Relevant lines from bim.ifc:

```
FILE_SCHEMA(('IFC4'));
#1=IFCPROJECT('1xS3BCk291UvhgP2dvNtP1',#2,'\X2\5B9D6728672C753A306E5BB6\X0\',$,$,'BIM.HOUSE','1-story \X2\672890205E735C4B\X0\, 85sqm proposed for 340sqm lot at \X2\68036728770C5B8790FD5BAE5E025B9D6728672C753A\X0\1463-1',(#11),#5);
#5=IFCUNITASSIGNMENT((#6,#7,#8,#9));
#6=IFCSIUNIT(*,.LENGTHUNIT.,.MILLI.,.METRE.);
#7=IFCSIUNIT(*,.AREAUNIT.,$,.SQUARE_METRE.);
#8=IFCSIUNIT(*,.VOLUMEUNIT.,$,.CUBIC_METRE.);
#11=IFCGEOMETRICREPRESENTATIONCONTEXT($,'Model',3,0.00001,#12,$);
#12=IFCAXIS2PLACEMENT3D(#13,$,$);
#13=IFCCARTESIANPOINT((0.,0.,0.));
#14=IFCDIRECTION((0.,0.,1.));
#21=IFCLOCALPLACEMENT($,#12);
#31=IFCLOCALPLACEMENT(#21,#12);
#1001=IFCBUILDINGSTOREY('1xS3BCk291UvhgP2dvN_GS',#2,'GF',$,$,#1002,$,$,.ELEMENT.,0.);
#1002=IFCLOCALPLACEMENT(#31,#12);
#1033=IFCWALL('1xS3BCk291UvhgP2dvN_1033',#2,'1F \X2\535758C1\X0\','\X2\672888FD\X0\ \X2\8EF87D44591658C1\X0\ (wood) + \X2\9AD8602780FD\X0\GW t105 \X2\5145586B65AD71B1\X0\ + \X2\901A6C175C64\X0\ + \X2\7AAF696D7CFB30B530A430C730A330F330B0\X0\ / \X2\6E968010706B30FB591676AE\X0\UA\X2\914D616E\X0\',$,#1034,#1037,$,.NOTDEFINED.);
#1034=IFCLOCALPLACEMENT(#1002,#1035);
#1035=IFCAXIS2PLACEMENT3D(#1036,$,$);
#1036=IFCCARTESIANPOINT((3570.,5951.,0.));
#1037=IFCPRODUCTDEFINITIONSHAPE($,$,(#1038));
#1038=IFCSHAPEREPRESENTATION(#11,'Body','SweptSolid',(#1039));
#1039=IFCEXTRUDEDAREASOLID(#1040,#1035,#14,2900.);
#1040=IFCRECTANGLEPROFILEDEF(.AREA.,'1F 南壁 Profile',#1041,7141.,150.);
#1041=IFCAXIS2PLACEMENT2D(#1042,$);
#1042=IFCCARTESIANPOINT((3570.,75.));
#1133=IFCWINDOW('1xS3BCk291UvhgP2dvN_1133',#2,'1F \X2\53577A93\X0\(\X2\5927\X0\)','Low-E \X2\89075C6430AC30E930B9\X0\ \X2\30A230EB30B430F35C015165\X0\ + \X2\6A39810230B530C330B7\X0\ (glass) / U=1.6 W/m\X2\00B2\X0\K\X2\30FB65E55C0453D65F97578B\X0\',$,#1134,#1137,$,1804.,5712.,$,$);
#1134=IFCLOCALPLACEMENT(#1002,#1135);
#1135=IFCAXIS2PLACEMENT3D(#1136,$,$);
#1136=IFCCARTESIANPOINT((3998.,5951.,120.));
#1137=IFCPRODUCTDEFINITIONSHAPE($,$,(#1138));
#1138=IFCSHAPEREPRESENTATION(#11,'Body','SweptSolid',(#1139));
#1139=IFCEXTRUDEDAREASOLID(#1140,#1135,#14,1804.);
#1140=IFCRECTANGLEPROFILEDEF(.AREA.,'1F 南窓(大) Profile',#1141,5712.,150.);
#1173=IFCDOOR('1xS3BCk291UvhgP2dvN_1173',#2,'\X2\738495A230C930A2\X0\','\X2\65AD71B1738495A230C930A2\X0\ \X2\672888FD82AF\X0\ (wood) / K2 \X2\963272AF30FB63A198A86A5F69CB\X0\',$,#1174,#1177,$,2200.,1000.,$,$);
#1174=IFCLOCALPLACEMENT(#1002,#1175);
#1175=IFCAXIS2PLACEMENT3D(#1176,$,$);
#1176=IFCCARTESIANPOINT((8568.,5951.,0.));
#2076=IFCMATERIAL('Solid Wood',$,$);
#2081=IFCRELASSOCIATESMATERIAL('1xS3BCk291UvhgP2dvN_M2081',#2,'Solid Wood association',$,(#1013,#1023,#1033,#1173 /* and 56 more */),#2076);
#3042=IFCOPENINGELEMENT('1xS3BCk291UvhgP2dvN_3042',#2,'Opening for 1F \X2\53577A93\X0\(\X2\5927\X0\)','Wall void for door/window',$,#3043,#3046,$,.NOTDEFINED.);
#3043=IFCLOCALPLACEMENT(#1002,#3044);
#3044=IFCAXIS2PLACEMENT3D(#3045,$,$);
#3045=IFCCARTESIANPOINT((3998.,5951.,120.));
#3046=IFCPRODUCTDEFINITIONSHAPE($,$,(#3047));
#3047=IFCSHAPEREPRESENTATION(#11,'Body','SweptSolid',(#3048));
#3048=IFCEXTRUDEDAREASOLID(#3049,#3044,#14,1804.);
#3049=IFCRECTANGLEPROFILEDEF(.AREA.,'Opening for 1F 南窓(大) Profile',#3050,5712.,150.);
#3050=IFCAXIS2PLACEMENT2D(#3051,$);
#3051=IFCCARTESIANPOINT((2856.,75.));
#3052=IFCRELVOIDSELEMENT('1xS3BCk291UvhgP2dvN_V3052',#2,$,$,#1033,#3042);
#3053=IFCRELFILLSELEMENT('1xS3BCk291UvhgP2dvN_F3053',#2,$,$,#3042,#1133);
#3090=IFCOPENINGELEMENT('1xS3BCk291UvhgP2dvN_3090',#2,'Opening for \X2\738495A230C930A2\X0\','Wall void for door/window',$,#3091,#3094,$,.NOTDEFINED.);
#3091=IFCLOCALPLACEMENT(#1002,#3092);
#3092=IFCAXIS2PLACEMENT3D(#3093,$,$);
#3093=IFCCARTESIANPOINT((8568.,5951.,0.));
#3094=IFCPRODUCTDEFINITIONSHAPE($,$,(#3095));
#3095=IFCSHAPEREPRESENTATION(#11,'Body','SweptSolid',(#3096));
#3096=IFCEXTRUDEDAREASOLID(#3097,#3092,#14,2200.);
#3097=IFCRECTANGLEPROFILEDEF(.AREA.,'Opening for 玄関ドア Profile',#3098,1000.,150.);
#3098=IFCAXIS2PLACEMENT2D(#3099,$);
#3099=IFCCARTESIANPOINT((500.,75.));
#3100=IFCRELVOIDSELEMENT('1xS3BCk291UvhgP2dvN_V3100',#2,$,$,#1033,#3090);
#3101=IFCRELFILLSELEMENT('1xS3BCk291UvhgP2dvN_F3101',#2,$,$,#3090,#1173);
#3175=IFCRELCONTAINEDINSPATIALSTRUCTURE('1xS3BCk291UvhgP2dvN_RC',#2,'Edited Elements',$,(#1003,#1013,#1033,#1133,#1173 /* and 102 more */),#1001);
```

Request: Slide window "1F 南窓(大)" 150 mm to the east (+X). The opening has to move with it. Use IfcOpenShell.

```python
import ifcopenshell
import ifcopenshell.api.geometry
import ifcopenshell.util.placement
import ifcopenshell.util.unit

model = ifcopenshell.open("bim.ifc")
unit_scale = ifcopenshell.util.unit.calculate_unit_scale(model)

window = model.by_id(1133)
opening = window.FillsVoids[0].RelatingOpeningElement
wall = opening.VoidsElements[0].RelatingBuildingElement

wall_matrix = ifcopenshell.util.placement.get_local_placement(wall.ObjectPlacement)
shift = wall_matrix[:3, 0] * 0.15 / unit_scale
before = ifcopenshell.util.placement.get_local_placement(window.ObjectPlacement)[:3, 3].copy()

# The window is not placed relative to its opening, so move both.
for product in (opening, window):
    matrix = ifcopenshell.util.placement.get_local_placement(product.ObjectPlacement)
    matrix[:3, 3] += shift
    ifcopenshell.api.geometry.edit_object_placement(model, product=product, matrix=matrix, is_si=False)

after = ifcopenshell.util.placement.get_local_placement(window.ObjectPlacement)[:3, 3]
print("window moved by", (after - before).round(3) + 0.0)

model.write("bim_edited.ifc")
```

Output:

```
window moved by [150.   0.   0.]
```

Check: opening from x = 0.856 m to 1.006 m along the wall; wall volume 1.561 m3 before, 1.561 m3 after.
